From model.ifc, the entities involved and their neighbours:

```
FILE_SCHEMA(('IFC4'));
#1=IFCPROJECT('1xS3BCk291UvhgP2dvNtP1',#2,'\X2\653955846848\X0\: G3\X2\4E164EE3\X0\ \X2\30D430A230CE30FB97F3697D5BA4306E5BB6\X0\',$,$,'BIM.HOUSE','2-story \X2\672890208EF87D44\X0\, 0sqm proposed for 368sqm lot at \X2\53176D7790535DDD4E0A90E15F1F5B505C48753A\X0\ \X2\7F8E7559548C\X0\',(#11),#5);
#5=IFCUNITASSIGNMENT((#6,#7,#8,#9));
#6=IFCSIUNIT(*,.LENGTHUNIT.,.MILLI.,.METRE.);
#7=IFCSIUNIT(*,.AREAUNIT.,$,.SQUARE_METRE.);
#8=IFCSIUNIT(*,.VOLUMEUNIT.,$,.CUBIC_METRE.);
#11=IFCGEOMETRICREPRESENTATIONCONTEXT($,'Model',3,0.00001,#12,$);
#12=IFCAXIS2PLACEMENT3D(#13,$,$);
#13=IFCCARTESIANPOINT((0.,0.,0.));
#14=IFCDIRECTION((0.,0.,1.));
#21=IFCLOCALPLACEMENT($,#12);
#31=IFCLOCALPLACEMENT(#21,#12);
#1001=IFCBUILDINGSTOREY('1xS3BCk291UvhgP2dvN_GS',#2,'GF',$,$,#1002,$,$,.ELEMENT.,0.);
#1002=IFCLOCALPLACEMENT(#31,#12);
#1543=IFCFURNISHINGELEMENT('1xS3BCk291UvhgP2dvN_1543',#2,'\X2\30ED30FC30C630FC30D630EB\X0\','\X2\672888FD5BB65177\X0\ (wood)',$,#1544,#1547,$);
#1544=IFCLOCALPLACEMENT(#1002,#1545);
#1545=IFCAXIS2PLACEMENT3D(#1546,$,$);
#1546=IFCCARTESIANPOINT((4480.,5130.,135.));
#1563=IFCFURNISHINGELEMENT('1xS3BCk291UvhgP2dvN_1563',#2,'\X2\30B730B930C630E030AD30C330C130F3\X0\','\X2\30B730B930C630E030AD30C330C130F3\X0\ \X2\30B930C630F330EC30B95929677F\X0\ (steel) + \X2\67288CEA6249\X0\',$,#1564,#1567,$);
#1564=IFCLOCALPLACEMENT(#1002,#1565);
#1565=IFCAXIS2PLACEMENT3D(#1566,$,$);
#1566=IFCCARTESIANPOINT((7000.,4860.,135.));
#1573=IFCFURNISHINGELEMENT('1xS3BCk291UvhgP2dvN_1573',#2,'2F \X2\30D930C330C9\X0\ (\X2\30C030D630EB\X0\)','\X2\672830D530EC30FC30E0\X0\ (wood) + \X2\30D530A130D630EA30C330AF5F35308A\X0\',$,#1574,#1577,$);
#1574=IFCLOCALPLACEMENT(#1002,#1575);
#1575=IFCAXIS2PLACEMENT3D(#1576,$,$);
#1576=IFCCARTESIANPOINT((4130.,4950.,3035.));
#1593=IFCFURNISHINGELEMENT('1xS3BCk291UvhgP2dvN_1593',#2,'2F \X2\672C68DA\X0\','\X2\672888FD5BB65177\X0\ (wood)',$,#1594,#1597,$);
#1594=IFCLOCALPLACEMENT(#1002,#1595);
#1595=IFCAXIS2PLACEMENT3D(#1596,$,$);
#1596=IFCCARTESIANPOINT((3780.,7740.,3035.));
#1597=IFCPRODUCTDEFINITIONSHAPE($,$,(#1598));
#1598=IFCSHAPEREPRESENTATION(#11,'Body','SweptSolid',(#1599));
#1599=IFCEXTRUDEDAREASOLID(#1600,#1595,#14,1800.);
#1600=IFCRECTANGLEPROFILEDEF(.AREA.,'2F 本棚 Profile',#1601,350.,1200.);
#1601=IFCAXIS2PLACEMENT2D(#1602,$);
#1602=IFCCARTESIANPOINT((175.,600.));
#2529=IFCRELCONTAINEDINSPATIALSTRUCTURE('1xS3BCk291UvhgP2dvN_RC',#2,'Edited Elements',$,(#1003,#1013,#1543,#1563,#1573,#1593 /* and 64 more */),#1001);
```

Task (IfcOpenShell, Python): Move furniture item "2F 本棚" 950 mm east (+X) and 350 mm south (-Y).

```python
import ifcopenshell
import ifcopenshell.api.geometry
import ifcopenshell.util.placement

model = ifcopenshell.open("model.ifc")

item = model.by_guid("1xS3BCk291UvhgP2dvN_1593")
matrix = ifcopenshell.util.placement.get_local_placement(item.ObjectPlacement)
matrix[0, 3] += 950.0
matrix[1, 3] -= 350.0
ifcopenshell.api.geometry.edit_object_placement(model, product=item, matrix=matrix, is_si=False)

print(ifcopenshell.util.placement.get_local_placement(item.ObjectPlacement).round(3) + 0.0)

model.write("model_updated.ifc")
```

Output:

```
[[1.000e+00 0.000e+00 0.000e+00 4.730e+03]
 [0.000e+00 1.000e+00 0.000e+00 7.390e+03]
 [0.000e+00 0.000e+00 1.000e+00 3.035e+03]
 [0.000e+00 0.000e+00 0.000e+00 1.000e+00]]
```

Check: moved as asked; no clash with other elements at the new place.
